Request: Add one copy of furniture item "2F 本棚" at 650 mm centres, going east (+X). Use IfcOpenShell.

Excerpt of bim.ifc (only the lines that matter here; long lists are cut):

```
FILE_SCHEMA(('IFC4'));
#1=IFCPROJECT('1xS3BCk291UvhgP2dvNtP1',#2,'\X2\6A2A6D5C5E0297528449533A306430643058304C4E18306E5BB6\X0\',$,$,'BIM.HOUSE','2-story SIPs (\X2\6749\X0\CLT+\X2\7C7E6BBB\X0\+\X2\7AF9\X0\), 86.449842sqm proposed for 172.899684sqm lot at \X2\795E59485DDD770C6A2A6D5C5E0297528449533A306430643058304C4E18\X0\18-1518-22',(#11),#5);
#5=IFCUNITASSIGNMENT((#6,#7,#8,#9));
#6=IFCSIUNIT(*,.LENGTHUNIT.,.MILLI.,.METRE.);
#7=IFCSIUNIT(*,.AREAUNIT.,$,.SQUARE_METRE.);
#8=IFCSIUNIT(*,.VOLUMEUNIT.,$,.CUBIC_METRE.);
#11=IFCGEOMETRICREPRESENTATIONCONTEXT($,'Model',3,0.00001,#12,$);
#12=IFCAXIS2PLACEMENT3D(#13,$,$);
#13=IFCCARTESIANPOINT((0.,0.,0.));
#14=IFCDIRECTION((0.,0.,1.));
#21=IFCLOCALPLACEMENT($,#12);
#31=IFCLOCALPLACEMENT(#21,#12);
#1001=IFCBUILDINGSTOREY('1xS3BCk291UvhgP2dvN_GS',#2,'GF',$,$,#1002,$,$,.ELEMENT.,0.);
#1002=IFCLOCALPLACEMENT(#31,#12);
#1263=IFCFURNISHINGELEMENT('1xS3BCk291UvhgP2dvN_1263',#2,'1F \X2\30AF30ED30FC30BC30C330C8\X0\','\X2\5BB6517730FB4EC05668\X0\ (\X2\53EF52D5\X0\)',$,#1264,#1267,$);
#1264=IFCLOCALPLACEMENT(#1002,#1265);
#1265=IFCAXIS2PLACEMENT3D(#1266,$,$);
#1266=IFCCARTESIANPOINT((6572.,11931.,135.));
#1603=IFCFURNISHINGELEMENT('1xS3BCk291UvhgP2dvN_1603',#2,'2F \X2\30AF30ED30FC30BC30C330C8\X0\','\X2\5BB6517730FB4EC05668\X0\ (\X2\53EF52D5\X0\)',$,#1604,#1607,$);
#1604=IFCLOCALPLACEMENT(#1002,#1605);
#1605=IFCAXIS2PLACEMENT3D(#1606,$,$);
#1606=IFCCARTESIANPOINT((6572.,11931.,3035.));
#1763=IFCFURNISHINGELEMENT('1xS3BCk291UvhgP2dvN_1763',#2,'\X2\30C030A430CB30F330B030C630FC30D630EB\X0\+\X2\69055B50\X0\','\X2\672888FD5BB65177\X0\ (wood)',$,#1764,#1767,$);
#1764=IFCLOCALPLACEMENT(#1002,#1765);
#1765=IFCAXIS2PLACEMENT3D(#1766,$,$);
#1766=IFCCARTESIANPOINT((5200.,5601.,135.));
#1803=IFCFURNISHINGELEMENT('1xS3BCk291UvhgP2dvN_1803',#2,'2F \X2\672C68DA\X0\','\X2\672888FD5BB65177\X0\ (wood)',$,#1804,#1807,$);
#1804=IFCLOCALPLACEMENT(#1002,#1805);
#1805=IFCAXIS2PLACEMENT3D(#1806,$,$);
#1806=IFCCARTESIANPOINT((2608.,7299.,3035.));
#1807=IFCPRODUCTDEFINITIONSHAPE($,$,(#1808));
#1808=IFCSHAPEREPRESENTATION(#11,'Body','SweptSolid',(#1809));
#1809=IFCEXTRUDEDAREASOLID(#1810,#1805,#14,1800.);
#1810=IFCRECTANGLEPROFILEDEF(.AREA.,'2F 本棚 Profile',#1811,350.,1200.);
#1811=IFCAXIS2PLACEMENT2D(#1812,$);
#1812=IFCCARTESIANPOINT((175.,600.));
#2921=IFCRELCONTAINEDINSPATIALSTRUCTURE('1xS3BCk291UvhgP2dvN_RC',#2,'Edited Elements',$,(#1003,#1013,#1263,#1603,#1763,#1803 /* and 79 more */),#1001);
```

```python
import numpy as np
import ifcopenshell
import ifcopenshell.api.geometry
import ifcopenshell.api.root
import ifcopenshell.util.element
import ifcopenshell.util.placement

model = ifcopenshell.open("bim.ifc")


def reuse_history(source, copy):
    """copy_class also copies each property set's owner history, people and application; keep the originals."""
    for rel in copy.IsDefinedBy:
        if rel.is_a("IfcRelDefinesByProperties") and (history := rel.RelatingPropertyDefinition.OwnerHistory):
            rel.RelatingPropertyDefinition.OwnerHistory = source.OwnerHistory
            ifcopenshell.util.element.remove_deep2(model, history)


source = model.by_id(1803)
base = ifcopenshell.util.placement.get_local_placement(source.ObjectPlacement)
step = np.array([1.0, 0.0, 0.0]) * 650.0

for i in range(1, 2):
    copy = ifcopenshell.api.root.copy_class(model, product=source)
    copy.Representation = ifcopenshell.util.element.copy_deep(
        model, source.Representation, exclude=["IfcGeometricRepresentationContext", "IfcRepresentationMap"]
    )
    reuse_history(source, copy)
    matrix = base.copy()
    matrix[:3, 3] += i * step
    print("added at", matrix[:3, 3].round(3) + 0.0)
    ifcopenshell.api.geometry.edit_object_placement(model, product=copy, matrix=matrix, is_si=False)

model.write("bim-out.ifc")
```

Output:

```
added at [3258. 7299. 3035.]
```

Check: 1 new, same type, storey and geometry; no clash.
